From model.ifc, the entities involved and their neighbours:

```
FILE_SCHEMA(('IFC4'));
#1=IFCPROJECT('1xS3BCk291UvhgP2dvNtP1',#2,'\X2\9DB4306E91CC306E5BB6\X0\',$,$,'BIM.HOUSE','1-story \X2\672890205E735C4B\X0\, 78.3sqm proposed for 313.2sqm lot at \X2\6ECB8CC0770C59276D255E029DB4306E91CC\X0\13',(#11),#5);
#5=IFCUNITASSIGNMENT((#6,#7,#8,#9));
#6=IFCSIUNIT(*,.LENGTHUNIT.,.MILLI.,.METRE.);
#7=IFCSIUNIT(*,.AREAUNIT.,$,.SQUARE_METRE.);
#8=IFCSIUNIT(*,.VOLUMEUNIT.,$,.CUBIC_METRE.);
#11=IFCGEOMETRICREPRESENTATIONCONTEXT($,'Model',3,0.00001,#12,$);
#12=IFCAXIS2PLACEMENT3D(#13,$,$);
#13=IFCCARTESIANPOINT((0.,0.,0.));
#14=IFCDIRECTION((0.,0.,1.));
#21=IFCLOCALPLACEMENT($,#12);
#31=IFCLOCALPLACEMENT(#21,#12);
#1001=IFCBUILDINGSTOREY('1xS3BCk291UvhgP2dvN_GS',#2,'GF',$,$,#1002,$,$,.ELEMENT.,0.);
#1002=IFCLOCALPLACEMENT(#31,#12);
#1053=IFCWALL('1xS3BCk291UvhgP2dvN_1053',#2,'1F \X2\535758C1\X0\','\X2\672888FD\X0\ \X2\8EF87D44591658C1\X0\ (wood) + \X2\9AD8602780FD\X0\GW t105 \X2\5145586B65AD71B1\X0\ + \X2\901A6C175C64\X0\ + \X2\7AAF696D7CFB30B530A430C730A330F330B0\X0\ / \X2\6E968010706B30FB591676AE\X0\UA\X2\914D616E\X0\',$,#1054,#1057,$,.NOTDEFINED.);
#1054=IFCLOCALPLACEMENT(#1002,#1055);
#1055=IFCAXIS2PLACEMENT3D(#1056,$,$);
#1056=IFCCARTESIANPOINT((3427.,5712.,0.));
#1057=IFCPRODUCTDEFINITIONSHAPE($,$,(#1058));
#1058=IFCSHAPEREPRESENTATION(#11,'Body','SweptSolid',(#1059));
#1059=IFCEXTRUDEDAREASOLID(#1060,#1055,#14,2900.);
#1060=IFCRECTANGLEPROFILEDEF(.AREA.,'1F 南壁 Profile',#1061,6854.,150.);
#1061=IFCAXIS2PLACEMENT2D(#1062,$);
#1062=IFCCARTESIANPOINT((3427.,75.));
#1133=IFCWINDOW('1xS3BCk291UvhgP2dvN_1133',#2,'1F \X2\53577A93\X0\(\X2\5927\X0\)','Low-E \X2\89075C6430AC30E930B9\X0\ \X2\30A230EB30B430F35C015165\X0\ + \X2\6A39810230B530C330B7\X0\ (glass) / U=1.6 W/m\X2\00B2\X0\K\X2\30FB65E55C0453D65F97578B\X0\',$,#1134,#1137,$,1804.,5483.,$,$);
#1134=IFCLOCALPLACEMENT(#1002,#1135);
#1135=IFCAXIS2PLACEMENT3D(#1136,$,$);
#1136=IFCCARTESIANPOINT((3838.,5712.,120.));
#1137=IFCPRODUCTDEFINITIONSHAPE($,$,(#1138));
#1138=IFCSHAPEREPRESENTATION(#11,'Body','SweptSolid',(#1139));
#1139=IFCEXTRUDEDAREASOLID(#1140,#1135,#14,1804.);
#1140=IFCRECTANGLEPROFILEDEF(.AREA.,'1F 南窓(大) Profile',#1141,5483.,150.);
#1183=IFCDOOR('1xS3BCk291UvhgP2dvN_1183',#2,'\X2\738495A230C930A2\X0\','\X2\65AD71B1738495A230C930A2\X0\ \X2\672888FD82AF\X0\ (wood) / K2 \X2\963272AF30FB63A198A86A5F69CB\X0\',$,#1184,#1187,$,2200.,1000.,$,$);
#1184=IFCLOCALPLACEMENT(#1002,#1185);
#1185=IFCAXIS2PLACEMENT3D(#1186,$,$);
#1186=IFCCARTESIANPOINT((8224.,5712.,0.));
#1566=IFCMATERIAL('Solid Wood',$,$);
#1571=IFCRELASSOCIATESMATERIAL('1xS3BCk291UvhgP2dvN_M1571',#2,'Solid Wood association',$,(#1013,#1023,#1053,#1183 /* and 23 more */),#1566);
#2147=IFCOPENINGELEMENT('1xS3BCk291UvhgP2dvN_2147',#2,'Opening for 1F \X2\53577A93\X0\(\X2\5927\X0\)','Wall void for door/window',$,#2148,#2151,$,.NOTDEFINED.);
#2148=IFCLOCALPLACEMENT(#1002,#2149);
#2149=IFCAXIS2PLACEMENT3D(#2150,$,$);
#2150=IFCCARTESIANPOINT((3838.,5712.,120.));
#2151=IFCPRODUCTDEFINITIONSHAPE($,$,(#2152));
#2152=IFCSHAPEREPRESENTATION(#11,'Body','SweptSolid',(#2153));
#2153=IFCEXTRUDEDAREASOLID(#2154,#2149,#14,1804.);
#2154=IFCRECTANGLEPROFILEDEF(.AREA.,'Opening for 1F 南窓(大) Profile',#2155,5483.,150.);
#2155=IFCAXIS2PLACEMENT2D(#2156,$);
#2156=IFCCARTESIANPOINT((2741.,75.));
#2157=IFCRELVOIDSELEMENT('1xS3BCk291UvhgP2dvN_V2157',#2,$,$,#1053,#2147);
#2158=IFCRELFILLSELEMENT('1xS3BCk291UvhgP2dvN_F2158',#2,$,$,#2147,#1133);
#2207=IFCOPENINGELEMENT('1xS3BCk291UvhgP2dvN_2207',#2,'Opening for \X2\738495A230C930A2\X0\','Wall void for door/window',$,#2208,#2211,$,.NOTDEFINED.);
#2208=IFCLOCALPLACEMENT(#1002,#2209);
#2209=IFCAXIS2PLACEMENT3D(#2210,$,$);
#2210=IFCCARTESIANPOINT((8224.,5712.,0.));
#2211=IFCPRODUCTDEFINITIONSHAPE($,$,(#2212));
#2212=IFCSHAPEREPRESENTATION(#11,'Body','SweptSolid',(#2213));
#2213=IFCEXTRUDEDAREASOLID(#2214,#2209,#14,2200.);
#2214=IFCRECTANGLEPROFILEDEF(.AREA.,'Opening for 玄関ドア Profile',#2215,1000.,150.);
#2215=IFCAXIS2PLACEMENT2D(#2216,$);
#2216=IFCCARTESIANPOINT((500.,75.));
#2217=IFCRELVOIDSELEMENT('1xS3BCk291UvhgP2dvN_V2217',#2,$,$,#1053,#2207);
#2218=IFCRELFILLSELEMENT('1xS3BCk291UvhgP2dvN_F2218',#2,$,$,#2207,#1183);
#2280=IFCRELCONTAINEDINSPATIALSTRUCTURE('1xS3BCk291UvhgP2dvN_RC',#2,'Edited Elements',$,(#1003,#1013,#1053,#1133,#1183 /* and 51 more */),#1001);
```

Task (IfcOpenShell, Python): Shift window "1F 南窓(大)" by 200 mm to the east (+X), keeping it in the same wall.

```python
import ifcopenshell
import ifcopenshell.api.geometry
import ifcopenshell.util.placement
import ifcopenshell.util.unit

model = ifcopenshell.open("model.ifc")
unit_scale = ifcopenshell.util.unit.calculate_unit_scale(model)

window = model.by_guid("1xS3BCk291UvhgP2dvN_1133")
opening = window.FillsVoids[0].RelatingOpeningElement
wall = opening.VoidsElements[0].RelatingBuildingElement

wall_matrix = ifcopenshell.util.placement.get_local_placement(wall.ObjectPlacement)
shift = wall_matrix[:3, 0] * 0.2 / unit_scale
before = ifcopenshell.util.placement.get_local_placement(window.ObjectPlacement)[:3, 3].copy()

# The window is not placed relative to its opening, so move both.
for product in (opening, window):
    matrix = ifcopenshell.util.placement.get_local_placement(product.ObjectPlacement)
    matrix[:3, 3] += shift
    ifcopenshell.api.geometry.edit_object_placement(model, product=product, matrix=matrix, is_si=False)

after = ifcopenshell.util.placement.get_local_placement(window.ObjectPlacement)[:3, 3]
print("window moved by", (after - before).round(3) + 0.0)

model.write("model-out.ifc")
```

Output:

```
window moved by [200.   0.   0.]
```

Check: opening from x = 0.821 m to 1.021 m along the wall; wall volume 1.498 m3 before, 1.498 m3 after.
